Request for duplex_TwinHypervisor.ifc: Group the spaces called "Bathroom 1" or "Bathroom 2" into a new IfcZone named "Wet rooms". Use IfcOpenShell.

First a look at what the model holds.

```python
import ifcopenshell

model = ifcopenshell.open("duplex_TwinHypervisor.ifc")
print(model.schema)
seen = {}
for space in model.by_type("IfcSpace"):
    seen[space.LongName] = seen.get(space.LongName, 0) + 1
for name, count in sorted(seen.items(), key=str):
    print(count, "x", name)
print("zones:", [z.Name for z in model.by_type("IfcZone")][:20])
```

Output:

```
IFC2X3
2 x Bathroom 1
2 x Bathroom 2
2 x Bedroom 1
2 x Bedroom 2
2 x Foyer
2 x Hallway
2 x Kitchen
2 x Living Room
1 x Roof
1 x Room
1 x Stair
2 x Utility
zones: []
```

```python
import ifcopenshell
import ifcopenshell.api.group
import ifcopenshell.api.root

model = ifcopenshell.open("duplex_TwinHypervisor.ifc")

names = {"Bathroom 1", "Bathroom 2"}
spaces = [s for s in model.by_type("IfcSpace") if s.LongName in names]

zone = ifcopenshell.api.root.create_entity(model, ifc_class="IfcZone", name="Wet rooms")
ifcopenshell.api.group.assign_group(model, products=spaces, group=zone)
print(len(spaces), "spaces in", zone.Name)

model.write("duplex_TwinHypervisor-out.ifc")
```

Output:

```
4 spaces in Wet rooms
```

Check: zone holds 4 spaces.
